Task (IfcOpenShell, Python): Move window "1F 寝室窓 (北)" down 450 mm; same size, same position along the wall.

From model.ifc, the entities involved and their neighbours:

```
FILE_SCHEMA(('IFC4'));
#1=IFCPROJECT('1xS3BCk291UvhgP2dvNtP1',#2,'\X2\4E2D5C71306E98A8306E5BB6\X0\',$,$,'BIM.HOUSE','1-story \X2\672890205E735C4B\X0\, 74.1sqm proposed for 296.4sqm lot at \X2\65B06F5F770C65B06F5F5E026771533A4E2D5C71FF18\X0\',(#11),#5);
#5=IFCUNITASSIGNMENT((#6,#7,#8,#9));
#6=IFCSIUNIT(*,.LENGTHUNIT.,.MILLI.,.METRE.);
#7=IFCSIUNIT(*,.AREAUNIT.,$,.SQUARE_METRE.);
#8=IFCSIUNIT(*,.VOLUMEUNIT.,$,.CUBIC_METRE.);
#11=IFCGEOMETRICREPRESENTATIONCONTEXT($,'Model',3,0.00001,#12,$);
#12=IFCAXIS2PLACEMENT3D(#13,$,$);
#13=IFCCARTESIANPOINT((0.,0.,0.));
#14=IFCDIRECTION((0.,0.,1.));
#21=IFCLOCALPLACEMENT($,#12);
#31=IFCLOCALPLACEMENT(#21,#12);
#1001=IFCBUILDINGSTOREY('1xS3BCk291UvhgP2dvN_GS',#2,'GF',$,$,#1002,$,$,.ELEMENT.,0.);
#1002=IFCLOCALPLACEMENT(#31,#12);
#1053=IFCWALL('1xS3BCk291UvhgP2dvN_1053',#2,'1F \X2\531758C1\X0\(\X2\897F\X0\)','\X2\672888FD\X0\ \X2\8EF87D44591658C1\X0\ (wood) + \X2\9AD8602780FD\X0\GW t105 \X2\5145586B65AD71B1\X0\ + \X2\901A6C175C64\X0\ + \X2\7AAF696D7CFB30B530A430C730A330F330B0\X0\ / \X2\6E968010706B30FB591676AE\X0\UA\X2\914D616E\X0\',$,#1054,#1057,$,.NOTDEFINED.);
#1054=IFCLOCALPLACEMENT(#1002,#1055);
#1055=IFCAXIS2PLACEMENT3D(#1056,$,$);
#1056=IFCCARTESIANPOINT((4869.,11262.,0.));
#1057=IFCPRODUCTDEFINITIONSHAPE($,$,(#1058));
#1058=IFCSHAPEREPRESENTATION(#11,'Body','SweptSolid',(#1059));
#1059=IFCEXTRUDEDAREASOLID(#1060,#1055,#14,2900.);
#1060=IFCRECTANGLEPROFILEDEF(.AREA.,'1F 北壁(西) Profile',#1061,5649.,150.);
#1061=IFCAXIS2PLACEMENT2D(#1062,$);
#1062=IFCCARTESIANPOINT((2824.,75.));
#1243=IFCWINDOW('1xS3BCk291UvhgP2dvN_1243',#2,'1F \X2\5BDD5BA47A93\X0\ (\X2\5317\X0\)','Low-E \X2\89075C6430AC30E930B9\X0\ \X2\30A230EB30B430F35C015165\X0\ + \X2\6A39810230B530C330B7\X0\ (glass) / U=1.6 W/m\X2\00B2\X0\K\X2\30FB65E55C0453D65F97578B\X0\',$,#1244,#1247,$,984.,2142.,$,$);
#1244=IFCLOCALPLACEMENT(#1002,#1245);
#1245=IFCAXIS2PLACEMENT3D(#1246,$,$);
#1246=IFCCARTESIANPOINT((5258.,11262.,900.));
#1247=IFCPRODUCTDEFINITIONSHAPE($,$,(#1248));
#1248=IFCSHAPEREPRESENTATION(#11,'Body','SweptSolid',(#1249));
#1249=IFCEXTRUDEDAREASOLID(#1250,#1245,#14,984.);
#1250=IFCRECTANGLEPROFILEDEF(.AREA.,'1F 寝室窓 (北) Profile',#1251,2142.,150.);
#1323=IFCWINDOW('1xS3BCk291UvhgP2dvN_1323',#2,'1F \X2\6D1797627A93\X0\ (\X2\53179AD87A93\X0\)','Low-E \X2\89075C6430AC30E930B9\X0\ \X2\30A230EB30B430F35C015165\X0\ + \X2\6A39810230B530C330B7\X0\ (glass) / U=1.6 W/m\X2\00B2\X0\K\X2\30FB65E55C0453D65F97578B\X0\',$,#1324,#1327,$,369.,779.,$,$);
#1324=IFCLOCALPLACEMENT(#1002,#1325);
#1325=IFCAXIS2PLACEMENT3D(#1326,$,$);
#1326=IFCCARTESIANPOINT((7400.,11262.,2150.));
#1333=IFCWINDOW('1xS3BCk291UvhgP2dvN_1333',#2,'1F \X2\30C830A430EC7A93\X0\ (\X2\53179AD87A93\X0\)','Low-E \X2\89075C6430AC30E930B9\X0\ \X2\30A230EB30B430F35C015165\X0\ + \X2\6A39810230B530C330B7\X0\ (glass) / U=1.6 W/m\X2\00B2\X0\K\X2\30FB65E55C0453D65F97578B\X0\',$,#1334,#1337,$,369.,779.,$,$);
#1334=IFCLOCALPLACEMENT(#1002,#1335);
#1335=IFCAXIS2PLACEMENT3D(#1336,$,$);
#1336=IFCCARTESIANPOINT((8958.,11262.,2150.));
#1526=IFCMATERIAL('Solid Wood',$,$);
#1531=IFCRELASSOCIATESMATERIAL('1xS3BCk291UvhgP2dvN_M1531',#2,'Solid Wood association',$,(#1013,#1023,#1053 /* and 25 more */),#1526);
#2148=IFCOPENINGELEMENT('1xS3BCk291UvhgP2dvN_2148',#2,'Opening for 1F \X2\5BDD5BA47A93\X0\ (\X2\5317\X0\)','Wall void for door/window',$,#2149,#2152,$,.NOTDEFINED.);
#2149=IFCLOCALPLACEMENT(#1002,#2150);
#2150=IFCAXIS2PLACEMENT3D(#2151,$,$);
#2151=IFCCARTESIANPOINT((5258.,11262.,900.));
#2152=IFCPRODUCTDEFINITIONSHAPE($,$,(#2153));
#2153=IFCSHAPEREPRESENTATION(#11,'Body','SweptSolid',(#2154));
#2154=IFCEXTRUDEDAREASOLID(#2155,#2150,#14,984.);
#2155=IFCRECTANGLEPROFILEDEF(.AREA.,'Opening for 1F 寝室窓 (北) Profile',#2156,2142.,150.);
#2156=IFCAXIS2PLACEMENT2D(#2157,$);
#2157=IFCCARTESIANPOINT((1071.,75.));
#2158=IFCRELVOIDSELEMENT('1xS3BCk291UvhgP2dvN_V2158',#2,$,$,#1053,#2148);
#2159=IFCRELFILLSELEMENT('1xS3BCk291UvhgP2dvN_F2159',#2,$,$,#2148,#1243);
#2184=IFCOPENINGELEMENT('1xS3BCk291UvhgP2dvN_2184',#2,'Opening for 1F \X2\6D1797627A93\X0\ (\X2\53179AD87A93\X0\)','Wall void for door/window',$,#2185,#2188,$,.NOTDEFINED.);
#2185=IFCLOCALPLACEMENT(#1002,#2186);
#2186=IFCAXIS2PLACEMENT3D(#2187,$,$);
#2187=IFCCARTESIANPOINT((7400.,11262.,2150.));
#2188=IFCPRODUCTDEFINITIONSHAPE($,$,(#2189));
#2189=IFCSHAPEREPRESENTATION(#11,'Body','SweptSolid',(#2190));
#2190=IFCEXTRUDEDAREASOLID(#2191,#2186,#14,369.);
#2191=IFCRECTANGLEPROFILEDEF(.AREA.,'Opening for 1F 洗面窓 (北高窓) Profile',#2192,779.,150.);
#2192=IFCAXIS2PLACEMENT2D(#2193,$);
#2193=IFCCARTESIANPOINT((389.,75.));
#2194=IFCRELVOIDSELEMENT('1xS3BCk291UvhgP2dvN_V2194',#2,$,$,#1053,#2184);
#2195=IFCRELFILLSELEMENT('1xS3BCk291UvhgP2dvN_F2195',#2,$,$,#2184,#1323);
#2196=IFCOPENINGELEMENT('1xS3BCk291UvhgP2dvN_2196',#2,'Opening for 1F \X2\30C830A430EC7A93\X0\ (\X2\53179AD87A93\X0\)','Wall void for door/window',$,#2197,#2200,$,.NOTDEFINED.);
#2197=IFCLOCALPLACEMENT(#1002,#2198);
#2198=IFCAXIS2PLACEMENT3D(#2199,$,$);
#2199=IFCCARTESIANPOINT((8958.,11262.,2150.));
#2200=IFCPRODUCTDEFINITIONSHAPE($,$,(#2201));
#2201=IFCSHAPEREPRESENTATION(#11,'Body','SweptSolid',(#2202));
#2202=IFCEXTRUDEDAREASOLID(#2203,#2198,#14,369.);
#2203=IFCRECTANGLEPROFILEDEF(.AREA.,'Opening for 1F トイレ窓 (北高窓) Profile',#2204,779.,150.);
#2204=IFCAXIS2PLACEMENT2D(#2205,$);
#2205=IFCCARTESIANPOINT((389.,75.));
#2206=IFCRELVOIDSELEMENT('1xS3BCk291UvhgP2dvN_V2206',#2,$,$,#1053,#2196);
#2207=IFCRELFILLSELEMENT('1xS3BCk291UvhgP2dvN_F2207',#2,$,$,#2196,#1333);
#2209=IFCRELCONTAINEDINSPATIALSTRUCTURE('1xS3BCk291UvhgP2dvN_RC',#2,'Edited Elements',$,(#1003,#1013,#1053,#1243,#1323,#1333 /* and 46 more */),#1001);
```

```python
import numpy as np
import ifcopenshell
import ifcopenshell.api.geometry
import ifcopenshell.util.placement
import ifcopenshell.util.unit

model = ifcopenshell.open("model.ifc")
unit_scale = ifcopenshell.util.unit.calculate_unit_scale(model)

window = model.by_id(1243)
opening = window.FillsVoids[0].RelatingOpeningElement
dz = -0.45 / unit_scale

shift = np.array([0.0, 0.0, dz])
# The window is not placed relative to its opening, so move both.
for product in (opening, window):
    matrix = ifcopenshell.util.placement.get_local_placement(product.ObjectPlacement)
    matrix[:3, 3] += shift
    ifcopenshell.api.geometry.edit_object_placement(model, product=product, matrix=matrix, is_si=False)

print(f"moved by {dz * unit_scale:+.3f} m")

model.write("model_v2.ifc")
```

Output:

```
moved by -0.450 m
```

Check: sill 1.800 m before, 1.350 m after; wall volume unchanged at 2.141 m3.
